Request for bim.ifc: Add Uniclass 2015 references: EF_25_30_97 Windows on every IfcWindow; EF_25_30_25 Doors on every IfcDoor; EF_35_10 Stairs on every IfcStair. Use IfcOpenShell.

First a look at what the model holds.

```python
import ifcopenshell

model = ifcopenshell.open("bim.ifc")
print(model.schema)
print("classifications:", [c.Name for c in model.by_type("IfcClassification")])
for ifc_class in ("IfcDoor", "IfcRoof", "IfcStair", "IfcWall", "IfcWindow"):
    print(ifc_class, len(model.by_type(ifc_class)))
```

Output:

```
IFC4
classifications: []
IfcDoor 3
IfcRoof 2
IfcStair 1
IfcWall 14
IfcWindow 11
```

```python
import ifcopenshell
import ifcopenshell.api.classification

model = ifcopenshell.open("bim.ifc")

system = ifcopenshell.api.classification.add_classification(model, classification="Uniclass 2015")

codes = {
    "IfcWindow": ("EF_25_30_97", "Windows"),
    "IfcDoor": ("EF_25_30_25", "Doors"),
    "IfcStair": ("EF_35_10", "Stairs"),
}
for ifc_class, (code, name) in codes.items():
    products = model.by_type(ifc_class)
    ifcopenshell.api.classification.add_reference(
        model, products=products, classification=system, identification=code, name=name
    )
    print(code, len(products))

model.write("bim_v2.ifc")
```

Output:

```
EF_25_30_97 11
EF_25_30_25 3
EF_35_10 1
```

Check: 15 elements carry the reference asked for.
